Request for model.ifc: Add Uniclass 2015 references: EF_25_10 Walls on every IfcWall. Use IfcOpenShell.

First a look at what the model holds.

```python
import ifcopenshell

model = ifcopenshell.open("model.ifc")
print(model.schema)
print("classifications:", [c.Name for c in model.by_type("IfcClassification")])
for ifc_class in ("IfcDoor", "IfcRoof", "IfcStair", "IfcWall", "IfcWindow"):
    print(ifc_class, len(model.by_type(ifc_class)))
```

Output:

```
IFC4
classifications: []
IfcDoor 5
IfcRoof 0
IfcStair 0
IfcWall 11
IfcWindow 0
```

```python
import ifcopenshell
import ifcopenshell.api.classification

model = ifcopenshell.open("model.ifc")

system = ifcopenshell.api.classification.add_classification(model, classification="Uniclass 2015")

codes = {
    "IfcWall": ("EF_25_10", "Walls"),
}
for ifc_class, (code, name) in codes.items():
    products = model.by_type(ifc_class)
    ifcopenshell.api.classification.add_reference(
        model, products=products, classification=system, identification=code, name=name
    )
    print(code, len(products))

model.write("model-out.ifc")
```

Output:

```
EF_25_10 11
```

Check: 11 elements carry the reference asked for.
